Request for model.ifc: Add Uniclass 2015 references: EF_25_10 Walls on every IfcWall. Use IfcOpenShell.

First a look at what the model holds.

```python
import ifcopenshell

model = ifcopenshell.open("model.ifc")
print(model.schema)
print("classifications:", [c.Name for c in model.by_type("IfcClassification")])
for ifc_class in ("IfcDoor", "IfcRoof", "IfcStair", "IfcWall", "IfcWindow"):
    print(ifc_class, len(model.by_type(ifc_class)))
```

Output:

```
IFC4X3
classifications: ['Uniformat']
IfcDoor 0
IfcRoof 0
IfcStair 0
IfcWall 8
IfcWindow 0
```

```python
import ifcopenshell
import ifcopenshell.api.classification

model = ifcopenshell.open("model.ifc")

system = ifcopenshell.api.classification.add_classification(model, classification="Uniclass 2015")

codes = {
    "IfcWall": ("EF_25_10", "Walls"),
}
for ifc_class, (code, name) in codes.items():
    products = model.by_type(ifc_class)
    ifcopenshell.api.classification.add_reference(
        model, products=products, classification=system, identification=code, name=name
    )
    print(code, len(products))

model.write("model_updated.ifc")
```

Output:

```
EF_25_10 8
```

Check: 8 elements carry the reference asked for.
